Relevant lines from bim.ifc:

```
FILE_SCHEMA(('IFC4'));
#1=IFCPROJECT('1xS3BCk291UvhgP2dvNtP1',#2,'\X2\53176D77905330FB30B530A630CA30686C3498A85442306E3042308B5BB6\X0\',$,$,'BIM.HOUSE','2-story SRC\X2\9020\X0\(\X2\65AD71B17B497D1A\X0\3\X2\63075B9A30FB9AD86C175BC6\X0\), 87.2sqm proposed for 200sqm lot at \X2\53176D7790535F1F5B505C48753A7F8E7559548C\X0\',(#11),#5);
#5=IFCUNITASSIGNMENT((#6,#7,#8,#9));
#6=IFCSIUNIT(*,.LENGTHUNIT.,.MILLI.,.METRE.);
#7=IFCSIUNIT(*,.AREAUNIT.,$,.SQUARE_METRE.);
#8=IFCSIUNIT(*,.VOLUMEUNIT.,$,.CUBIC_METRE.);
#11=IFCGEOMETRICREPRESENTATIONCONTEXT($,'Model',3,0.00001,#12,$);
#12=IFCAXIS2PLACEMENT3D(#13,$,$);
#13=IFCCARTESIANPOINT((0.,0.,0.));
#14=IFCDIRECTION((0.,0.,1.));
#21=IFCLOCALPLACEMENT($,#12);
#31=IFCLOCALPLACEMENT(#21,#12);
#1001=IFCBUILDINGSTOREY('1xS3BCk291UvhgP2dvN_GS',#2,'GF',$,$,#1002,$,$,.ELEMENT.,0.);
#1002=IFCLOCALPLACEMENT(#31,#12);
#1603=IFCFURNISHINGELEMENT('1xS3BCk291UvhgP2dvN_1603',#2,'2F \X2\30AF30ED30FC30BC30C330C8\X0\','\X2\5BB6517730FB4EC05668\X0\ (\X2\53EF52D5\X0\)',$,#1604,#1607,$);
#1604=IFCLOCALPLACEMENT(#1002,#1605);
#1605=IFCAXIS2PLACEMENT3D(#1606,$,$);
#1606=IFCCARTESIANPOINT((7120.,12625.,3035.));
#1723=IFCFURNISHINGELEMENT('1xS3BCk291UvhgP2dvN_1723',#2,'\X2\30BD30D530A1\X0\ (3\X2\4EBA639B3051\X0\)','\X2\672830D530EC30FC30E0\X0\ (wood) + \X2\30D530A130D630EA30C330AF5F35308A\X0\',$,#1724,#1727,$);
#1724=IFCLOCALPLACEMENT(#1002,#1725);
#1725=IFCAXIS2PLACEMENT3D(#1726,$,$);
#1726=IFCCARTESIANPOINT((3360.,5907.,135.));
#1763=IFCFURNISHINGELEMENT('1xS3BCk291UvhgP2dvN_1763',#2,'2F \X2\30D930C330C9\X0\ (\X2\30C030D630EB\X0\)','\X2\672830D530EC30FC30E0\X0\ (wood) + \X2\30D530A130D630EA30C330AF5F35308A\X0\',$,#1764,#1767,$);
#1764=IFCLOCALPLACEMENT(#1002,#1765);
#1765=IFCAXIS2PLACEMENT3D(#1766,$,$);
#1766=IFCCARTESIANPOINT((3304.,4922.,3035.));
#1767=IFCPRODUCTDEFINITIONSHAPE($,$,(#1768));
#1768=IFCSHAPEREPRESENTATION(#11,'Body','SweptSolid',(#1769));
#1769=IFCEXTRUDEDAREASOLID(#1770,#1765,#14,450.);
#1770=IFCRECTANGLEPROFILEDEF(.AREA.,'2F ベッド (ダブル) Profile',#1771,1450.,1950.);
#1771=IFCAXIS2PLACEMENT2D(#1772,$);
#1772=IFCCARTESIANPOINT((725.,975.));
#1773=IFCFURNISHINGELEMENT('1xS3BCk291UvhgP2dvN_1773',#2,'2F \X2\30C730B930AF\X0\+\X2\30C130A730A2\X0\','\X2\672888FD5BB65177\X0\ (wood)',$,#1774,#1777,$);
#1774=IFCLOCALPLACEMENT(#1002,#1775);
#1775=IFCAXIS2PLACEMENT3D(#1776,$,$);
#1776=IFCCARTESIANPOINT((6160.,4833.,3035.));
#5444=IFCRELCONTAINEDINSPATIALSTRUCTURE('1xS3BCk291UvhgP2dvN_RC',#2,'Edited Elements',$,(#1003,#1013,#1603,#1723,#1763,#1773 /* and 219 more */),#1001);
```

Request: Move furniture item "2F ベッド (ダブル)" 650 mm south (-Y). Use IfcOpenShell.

```python
import ifcopenshell
import ifcopenshell.api.geometry
import ifcopenshell.util.placement
import ifcopenshell.util.unit

model = ifcopenshell.open("bim.ifc")
unit_scale = ifcopenshell.util.unit.calculate_unit_scale(model)

item = model.by_guid("1xS3BCk291UvhgP2dvN_1763")
matrix = ifcopenshell.util.placement.get_local_placement(item.ObjectPlacement)
matrix[1, 3] -= 0.65 / unit_scale
ifcopenshell.api.geometry.edit_object_placement(model, product=item, matrix=matrix, is_si=False)

print(ifcopenshell.util.placement.get_local_placement(item.ObjectPlacement).round(3) + 0.0)

model.write("bim_edited.ifc")
```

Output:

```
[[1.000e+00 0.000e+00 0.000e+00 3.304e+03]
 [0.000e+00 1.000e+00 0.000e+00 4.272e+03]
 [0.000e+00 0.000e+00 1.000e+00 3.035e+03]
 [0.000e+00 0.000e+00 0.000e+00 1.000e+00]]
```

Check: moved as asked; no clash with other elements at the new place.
